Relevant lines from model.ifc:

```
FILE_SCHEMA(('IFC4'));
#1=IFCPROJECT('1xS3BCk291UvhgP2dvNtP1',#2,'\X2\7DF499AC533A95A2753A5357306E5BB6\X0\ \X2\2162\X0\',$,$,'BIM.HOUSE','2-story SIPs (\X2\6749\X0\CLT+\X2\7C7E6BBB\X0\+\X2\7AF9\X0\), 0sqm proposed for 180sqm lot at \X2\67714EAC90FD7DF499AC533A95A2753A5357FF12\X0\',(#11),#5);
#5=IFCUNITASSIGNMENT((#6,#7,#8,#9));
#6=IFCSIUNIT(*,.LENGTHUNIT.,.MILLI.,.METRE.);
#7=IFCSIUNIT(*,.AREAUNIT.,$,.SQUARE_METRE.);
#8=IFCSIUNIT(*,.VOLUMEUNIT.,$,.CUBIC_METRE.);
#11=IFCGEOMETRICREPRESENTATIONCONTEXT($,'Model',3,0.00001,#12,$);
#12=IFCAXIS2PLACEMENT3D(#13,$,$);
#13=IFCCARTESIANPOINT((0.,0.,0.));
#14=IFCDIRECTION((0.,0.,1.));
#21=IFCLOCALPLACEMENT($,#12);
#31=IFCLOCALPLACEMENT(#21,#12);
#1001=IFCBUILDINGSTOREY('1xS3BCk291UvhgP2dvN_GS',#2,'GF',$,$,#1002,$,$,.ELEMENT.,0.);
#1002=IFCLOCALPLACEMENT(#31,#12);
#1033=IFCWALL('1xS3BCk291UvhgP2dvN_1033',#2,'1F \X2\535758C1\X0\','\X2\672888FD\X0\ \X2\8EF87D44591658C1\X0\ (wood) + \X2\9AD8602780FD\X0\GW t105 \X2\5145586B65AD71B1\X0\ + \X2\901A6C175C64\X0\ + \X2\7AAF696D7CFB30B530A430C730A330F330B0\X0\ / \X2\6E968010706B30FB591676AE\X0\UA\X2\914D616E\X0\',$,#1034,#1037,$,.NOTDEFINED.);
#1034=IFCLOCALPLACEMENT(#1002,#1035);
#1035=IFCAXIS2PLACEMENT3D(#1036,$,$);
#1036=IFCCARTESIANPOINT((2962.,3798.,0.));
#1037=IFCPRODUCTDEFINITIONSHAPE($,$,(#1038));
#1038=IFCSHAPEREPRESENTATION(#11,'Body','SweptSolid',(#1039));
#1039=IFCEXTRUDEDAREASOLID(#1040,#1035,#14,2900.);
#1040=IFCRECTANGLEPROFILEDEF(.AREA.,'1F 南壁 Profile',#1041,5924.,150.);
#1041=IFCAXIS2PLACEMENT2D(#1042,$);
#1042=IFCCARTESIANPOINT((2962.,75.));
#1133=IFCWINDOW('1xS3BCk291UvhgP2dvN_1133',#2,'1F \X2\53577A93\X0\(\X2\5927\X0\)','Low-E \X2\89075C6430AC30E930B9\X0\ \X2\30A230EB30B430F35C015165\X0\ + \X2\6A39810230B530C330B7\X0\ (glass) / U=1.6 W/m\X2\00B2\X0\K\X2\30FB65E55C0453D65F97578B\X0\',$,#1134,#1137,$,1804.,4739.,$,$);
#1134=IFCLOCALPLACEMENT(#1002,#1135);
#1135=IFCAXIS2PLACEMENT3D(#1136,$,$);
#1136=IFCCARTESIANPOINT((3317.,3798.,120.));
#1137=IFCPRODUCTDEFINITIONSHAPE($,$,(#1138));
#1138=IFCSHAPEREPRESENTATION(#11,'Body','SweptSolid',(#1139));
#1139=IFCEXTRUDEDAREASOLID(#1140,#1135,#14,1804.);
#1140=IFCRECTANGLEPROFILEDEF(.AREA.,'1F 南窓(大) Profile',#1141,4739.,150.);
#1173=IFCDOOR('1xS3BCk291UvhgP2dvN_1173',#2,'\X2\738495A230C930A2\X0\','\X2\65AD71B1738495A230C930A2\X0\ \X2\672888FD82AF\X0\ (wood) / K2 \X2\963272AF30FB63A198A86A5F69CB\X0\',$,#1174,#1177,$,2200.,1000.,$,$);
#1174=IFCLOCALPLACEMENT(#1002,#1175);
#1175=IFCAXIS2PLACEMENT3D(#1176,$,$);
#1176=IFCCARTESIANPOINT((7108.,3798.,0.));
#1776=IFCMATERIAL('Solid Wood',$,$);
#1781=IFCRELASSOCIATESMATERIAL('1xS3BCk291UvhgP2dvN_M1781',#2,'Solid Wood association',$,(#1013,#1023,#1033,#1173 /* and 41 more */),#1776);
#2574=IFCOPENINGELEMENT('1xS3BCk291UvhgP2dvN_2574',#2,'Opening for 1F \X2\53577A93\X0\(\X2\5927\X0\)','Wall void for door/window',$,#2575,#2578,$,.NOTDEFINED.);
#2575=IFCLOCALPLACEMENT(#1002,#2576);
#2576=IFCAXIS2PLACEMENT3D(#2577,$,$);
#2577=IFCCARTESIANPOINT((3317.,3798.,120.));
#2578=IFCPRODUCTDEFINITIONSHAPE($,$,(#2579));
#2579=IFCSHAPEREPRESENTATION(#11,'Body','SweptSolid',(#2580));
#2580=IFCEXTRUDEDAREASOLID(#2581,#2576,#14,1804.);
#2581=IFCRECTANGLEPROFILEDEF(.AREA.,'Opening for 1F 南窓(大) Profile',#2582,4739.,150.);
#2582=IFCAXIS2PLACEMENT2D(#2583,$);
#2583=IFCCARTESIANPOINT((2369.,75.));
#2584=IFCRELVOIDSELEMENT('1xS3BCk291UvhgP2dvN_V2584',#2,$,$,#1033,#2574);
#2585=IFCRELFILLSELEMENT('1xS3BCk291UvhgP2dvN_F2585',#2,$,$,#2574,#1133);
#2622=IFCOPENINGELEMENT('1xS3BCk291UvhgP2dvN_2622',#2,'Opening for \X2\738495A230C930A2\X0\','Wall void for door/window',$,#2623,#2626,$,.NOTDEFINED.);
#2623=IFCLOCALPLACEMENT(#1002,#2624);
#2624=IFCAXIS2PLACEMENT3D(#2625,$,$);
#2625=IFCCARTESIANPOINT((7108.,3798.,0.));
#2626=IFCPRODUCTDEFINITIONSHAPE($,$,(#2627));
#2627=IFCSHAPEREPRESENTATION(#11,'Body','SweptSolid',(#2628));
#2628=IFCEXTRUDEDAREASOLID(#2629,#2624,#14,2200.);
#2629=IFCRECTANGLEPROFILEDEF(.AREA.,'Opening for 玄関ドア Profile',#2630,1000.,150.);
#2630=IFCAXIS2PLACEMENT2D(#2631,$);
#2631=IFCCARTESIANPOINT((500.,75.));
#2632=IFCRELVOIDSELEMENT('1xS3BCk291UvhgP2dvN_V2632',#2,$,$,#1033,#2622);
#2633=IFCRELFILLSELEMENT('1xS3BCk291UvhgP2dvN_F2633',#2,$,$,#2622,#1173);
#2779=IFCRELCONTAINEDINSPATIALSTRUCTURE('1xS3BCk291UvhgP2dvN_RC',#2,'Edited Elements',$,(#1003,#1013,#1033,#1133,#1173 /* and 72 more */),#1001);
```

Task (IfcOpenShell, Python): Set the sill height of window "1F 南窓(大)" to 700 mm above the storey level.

```python
import numpy as np
import ifcopenshell
import ifcopenshell.api.geometry
import ifcopenshell.geom
import ifcopenshell.util.element
import ifcopenshell.util.placement
import ifcopenshell.util.shape
import ifcopenshell.util.unit

model = ifcopenshell.open("model.ifc")
unit_scale = ifcopenshell.util.unit.calculate_unit_scale(model)

window = model.by_guid("1xS3BCk291UvhgP2dvN_1133")
opening = window.FillsVoids[0].RelatingOpeningElement
storey = ifcopenshell.util.element.get_container(window, ifc_class="IfcBuildingStorey")
level = ifcopenshell.util.placement.get_local_placement(storey.ObjectPlacement)[2, 3]

# The opening's origin need not be at the sill, so measure its lowest point.
shape = ifcopenshell.geom.create_shape(ifcopenshell.geom.settings(), opening)
bottom = ifcopenshell.util.shape.get_shape_bottom_elevation(shape, shape.geometry) / unit_scale
dz = level + 700.0 - bottom

shift = np.array([0.0, 0.0, dz])
# The window is not placed relative to its opening, so move both.
for product in (opening, window):
    matrix = ifcopenshell.util.placement.get_local_placement(product.ObjectPlacement)
    matrix[:3, 3] += shift
    ifcopenshell.api.geometry.edit_object_placement(model, product=product, matrix=matrix, is_si=False)

print(f"moved by {dz * unit_scale:+.3f} m")

model.write("model_v2.ifc")
```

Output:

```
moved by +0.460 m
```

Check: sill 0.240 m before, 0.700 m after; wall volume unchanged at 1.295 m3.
